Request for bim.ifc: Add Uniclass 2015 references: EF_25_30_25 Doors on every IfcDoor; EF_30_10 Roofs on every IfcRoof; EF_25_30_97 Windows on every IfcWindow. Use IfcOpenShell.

First a look at what the model holds.

```python
import ifcopenshell

model = ifcopenshell.open("bim.ifc")
print(model.schema)
print("classifications:", [c.Name for c in model.by_type("IfcClassification")])
for ifc_class in ("IfcDoor", "IfcRoof", "IfcStair", "IfcWall", "IfcWindow"):
    print(ifc_class, len(model.by_type(ifc_class)))
```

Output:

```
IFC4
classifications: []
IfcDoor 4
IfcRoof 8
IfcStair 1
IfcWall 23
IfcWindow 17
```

```python
import ifcopenshell
import ifcopenshell.api.classification

model = ifcopenshell.open("bim.ifc")

system = ifcopenshell.api.classification.add_classification(model, classification="Uniclass 2015")

codes = {
    "IfcDoor": ("EF_25_30_25", "Doors"),
    "IfcRoof": ("EF_30_10", "Roofs"),
    "IfcWindow": ("EF_25_30_97", "Windows"),
}
for ifc_class, (code, name) in codes.items():
    products = model.by_type(ifc_class)
    ifcopenshell.api.classification.add_reference(
        model, products=products, classification=system, identification=code, name=name
    )
    print(code, len(products))

model.write("bim_updated.ifc")
```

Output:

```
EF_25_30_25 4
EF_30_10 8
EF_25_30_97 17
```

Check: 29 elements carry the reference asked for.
